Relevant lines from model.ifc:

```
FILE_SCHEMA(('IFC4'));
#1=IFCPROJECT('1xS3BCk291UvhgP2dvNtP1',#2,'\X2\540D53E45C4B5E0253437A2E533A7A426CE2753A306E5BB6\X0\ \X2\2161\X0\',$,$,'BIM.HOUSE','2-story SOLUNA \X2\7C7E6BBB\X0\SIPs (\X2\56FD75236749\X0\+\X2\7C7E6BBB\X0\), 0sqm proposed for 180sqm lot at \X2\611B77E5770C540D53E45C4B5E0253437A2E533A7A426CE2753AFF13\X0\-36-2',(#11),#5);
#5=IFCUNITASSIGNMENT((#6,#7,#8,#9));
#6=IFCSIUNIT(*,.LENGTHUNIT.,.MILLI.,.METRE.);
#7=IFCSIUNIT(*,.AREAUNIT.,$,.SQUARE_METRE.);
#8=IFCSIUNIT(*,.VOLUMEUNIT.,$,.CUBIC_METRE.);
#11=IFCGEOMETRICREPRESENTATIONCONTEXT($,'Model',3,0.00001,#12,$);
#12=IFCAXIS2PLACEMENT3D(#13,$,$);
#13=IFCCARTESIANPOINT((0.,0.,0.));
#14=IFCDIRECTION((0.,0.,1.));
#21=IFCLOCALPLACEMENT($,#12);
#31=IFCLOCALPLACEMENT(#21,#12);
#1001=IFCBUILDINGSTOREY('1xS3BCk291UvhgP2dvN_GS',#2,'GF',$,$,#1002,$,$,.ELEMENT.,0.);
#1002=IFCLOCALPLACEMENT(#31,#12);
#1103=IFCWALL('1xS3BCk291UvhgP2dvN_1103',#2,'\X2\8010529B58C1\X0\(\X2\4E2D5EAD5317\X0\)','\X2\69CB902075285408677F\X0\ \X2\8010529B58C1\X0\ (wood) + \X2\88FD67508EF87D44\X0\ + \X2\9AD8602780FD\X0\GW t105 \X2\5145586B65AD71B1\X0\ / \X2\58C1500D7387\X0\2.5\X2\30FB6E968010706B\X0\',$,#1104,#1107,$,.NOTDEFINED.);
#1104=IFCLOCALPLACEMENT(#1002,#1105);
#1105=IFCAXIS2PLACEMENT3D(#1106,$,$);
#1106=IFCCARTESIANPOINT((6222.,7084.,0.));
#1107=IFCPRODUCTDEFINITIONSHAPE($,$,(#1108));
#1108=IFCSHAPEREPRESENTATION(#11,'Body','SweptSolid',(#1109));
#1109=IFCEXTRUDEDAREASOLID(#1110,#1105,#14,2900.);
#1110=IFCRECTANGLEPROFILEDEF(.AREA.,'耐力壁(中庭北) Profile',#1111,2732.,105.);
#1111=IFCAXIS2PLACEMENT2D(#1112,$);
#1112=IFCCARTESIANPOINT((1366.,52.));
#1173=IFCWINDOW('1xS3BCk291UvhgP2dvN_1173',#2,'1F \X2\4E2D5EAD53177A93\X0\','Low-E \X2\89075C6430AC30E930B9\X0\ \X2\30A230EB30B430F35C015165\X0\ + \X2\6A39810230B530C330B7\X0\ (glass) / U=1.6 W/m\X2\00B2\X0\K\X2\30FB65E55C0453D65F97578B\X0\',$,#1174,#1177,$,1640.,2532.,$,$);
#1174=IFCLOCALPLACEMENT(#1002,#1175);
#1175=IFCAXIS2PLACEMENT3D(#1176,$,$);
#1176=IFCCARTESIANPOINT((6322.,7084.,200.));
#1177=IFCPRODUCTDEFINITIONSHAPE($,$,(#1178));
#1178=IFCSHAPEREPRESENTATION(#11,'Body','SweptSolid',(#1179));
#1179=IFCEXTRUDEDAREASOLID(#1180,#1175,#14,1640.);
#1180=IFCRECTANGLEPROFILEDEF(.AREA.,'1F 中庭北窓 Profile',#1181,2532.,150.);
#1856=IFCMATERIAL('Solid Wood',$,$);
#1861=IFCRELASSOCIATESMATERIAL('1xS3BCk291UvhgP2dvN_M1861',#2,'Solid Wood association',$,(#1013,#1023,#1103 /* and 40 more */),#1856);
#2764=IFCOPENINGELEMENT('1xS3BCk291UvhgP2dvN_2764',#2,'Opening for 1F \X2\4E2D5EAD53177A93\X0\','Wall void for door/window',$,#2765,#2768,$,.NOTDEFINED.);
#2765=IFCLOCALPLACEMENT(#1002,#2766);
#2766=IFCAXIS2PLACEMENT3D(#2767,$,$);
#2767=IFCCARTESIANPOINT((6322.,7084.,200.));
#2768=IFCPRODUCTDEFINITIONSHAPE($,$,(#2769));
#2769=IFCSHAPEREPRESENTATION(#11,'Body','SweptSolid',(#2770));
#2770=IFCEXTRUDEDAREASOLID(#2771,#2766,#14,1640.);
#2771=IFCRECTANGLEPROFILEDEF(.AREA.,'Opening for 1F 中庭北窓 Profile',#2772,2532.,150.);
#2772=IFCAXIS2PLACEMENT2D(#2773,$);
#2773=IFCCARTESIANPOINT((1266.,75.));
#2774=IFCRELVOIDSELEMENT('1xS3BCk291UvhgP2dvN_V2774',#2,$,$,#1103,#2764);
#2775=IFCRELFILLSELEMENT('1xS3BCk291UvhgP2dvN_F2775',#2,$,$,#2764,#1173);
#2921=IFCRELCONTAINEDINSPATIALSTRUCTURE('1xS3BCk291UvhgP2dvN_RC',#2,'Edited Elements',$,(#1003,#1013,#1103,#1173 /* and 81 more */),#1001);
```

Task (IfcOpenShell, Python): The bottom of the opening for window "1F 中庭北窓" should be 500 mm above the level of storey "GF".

```python
import numpy as np
import ifcopenshell
import ifcopenshell.api.geometry
import ifcopenshell.geom
import ifcopenshell.util.element
import ifcopenshell.util.placement
import ifcopenshell.util.shape
import ifcopenshell.util.unit

model = ifcopenshell.open("model.ifc")
unit_scale = ifcopenshell.util.unit.calculate_unit_scale(model)

window = model.by_id(1173)
opening = window.FillsVoids[0].RelatingOpeningElement
storey = ifcopenshell.util.element.get_container(window, ifc_class="IfcBuildingStorey")
level = ifcopenshell.util.placement.get_local_placement(storey.ObjectPlacement)[2, 3]

# The opening's origin need not be at the sill, so measure its lowest point.
shape = ifcopenshell.geom.create_shape(ifcopenshell.geom.settings(), opening)
bottom = ifcopenshell.util.shape.get_shape_bottom_elevation(shape, shape.geometry) / unit_scale
dz = level + 0.5 / unit_scale - bottom

shift = np.array([0.0, 0.0, dz])
# The window is not placed relative to its opening, so move both.
for product in (opening, window):
    matrix = ifcopenshell.util.placement.get_local_placement(product.ObjectPlacement)
    matrix[:3, 3] += shift
    ifcopenshell.api.geometry.edit_object_placement(model, product=product, matrix=matrix, is_si=False)

print(f"moved by {dz * unit_scale:+.3f} m")

model.write("model-out.ifc")
```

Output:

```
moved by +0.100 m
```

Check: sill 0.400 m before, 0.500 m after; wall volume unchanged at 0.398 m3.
